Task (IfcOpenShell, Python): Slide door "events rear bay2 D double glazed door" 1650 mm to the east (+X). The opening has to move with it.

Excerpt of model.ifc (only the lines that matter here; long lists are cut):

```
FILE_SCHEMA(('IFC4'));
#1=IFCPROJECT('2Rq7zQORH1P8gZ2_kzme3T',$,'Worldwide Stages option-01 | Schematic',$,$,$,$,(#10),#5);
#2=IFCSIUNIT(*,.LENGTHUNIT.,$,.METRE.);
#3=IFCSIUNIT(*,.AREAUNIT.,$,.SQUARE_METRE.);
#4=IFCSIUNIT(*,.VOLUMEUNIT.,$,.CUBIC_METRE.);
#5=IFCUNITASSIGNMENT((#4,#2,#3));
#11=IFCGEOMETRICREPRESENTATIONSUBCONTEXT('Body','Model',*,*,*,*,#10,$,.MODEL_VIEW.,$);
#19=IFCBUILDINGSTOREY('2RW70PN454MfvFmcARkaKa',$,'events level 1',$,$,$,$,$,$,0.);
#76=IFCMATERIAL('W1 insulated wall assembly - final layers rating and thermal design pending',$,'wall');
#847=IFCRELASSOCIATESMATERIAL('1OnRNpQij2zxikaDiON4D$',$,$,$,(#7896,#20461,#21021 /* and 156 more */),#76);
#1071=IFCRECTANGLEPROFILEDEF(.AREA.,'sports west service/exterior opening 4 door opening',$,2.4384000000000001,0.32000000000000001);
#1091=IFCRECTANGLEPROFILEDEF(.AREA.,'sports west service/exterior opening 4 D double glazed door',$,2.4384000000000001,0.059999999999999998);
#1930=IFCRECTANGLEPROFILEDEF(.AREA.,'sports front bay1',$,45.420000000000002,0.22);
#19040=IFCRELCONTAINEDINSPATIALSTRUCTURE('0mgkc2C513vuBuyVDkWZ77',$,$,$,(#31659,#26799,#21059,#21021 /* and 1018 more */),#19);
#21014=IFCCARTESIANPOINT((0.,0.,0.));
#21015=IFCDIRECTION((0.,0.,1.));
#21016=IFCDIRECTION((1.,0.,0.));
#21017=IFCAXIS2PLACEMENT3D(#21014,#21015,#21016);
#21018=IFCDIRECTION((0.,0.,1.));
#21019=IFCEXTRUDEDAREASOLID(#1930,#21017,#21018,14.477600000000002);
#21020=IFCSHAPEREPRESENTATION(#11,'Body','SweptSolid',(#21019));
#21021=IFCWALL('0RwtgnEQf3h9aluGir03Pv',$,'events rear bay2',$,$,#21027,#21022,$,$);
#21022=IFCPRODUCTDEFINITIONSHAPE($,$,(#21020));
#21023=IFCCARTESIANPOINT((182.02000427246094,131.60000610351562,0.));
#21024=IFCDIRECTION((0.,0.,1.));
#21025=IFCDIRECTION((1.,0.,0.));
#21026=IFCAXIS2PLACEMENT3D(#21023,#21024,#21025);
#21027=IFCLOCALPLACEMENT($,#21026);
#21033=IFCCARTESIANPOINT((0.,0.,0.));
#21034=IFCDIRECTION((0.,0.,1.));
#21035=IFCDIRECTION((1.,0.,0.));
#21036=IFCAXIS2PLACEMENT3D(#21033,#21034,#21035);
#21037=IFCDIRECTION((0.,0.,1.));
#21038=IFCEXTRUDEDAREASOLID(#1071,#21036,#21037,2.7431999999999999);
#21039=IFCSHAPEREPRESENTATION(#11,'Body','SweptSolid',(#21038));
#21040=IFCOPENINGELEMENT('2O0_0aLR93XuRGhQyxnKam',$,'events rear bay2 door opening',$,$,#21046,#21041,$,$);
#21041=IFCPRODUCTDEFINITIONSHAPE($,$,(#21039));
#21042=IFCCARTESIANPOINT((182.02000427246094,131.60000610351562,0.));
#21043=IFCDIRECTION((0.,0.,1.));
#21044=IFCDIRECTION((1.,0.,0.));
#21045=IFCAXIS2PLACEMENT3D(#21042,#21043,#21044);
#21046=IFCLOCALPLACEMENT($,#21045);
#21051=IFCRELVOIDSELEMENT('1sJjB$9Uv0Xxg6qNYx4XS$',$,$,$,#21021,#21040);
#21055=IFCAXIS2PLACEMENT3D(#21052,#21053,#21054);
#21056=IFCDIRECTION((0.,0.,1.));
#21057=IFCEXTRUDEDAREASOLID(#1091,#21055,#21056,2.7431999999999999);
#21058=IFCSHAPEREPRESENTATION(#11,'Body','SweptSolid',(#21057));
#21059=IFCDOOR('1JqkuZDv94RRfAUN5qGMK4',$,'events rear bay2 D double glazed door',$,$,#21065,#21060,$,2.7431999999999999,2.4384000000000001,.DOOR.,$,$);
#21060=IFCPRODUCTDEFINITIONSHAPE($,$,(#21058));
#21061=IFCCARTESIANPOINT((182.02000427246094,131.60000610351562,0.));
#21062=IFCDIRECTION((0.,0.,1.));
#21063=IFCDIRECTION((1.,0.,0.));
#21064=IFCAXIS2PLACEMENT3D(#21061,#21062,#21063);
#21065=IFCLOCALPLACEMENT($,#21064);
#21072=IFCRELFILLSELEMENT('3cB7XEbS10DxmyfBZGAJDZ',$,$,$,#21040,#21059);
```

```python
import ifcopenshell
import ifcopenshell.api.geometry
import ifcopenshell.util.placement

model = ifcopenshell.open("model.ifc")

door = model.by_id(21059)
opening = door.FillsVoids[0].RelatingOpeningElement
wall = opening.VoidsElements[0].RelatingBuildingElement

wall_matrix = ifcopenshell.util.placement.get_local_placement(wall.ObjectPlacement)
shift = wall_matrix[:3, 0] * 1.65
before = ifcopenshell.util.placement.get_local_placement(door.ObjectPlacement)[:3, 3].copy()

# The door is not placed relative to its opening, so move both.
for product in (opening, door):
    matrix = ifcopenshell.util.placement.get_local_placement(product.ObjectPlacement)
    matrix[:3, 3] += shift
    ifcopenshell.api.geometry.edit_object_placement(model, product=product, matrix=matrix, is_si=False)

after = ifcopenshell.util.placement.get_local_placement(door.ObjectPlacement)[:3, 3]
print("door moved by", (after - before).round(3) + 0.0)

model.write("model_v2.ifc")
```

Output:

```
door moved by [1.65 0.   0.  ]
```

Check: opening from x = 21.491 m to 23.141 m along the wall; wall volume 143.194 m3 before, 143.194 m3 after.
